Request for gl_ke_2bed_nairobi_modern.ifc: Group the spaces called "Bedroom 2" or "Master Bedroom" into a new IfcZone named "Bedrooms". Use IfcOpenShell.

First a look at what the model holds.

```python
import ifcopenshell

model = ifcopenshell.open("gl_ke_2bed_nairobi_modern.ifc")
print(model.schema)
seen = {}
for space in model.by_type("IfcSpace"):
    seen[space.LongName] = seen.get(space.LongName, 0) + 1
for name, count in sorted(seen.items(), key=str):
    print(count, "x", name)
print("zones:", [z.Name for z in model.by_type("IfcZone")][:20])
```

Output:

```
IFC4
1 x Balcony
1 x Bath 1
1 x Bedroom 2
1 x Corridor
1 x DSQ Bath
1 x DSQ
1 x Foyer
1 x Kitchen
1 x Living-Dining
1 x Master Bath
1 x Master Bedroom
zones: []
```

```python
import ifcopenshell
import ifcopenshell.api.group
import ifcopenshell.api.root

model = ifcopenshell.open("gl_ke_2bed_nairobi_modern.ifc")

names = {"Bedroom 2", "Master Bedroom"}
spaces = [s for s in model.by_type("IfcSpace") if s.LongName in names]

zone = ifcopenshell.api.root.create_entity(model, ifc_class="IfcZone", name="Bedrooms")
ifcopenshell.api.group.assign_group(model, products=spaces, group=zone)
print(len(spaces), "spaces in", zone.Name)

model.write("gl_ke_2bed_nairobi_modern_v2.ifc")
```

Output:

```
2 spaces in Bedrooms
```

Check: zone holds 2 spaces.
